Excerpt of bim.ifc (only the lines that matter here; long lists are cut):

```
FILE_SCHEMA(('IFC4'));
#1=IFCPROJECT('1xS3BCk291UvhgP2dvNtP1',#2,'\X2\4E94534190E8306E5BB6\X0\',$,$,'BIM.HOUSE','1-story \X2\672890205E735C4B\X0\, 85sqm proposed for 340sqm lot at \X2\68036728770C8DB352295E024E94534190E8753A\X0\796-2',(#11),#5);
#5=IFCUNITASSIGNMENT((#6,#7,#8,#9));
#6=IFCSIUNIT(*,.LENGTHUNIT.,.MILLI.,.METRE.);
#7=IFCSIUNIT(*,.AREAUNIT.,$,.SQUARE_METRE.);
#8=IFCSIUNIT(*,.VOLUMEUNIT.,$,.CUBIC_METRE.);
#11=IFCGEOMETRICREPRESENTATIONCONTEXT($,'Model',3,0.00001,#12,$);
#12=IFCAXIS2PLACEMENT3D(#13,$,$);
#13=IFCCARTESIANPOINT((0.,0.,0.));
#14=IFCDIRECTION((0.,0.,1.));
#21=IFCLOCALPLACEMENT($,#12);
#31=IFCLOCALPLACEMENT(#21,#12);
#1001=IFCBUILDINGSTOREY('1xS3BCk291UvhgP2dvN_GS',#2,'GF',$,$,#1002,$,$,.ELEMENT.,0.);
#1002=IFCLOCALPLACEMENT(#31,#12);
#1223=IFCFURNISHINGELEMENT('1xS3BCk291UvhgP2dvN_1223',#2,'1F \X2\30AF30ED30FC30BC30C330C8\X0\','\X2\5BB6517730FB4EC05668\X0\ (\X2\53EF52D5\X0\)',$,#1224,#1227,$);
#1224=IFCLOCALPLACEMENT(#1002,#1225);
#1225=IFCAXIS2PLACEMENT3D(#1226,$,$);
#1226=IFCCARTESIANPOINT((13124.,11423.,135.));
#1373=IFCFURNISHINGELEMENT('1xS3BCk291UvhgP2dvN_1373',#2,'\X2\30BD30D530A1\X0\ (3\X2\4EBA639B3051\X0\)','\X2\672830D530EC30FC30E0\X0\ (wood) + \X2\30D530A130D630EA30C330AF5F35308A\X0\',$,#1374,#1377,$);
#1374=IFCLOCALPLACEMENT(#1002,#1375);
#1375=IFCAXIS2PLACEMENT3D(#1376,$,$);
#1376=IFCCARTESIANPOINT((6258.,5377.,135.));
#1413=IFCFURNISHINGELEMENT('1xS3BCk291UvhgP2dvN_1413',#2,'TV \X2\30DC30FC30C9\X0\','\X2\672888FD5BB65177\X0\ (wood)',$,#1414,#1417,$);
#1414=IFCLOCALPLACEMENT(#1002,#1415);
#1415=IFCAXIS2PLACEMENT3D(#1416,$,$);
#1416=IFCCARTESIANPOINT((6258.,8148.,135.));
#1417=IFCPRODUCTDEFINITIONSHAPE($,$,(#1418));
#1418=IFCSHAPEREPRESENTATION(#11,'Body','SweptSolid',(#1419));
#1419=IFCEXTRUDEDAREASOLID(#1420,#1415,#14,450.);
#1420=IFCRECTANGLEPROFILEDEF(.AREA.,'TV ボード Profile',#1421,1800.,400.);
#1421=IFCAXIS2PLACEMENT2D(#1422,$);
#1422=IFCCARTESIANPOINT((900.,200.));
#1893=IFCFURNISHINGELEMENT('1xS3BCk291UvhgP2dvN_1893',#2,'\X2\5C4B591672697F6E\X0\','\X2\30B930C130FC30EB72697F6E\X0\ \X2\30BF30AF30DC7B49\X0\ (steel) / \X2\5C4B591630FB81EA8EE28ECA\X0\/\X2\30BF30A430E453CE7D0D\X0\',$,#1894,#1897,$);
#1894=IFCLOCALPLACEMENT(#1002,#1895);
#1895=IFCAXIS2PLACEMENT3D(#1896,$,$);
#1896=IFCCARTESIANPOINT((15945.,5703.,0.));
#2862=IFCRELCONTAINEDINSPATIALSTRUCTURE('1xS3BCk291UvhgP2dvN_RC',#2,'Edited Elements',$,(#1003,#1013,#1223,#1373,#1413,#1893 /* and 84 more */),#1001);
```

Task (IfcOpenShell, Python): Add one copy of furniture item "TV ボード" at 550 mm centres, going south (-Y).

```python
import numpy as np
import ifcopenshell
import ifcopenshell.api.geometry
import ifcopenshell.api.root
import ifcopenshell.util.element
import ifcopenshell.util.placement
import ifcopenshell.util.unit

model = ifcopenshell.open("bim.ifc")
unit_scale = ifcopenshell.util.unit.calculate_unit_scale(model)


def reuse_history(source, copy):
    """copy_class also copies each property set's owner history, people and application; keep the originals."""
    for rel in copy.IsDefinedBy:
        if rel.is_a("IfcRelDefinesByProperties") and (history := rel.RelatingPropertyDefinition.OwnerHistory):
            rel.RelatingPropertyDefinition.OwnerHistory = source.OwnerHistory
            ifcopenshell.util.element.remove_deep2(model, history)


source = model.by_guid("1xS3BCk291UvhgP2dvN_1413")
base = ifcopenshell.util.placement.get_local_placement(source.ObjectPlacement)
step = np.array([0.0, -1.0, 0.0]) * 0.55 / unit_scale

for i in range(1, 2):
    copy = ifcopenshell.api.root.copy_class(model, product=source)
    copy.Representation = ifcopenshell.util.element.copy_deep(
        model, source.Representation, exclude=["IfcGeometricRepresentationContext", "IfcRepresentationMap"]
    )
    reuse_history(source, copy)
    matrix = base.copy()
    matrix[:3, 3] += i * step
    print("added at", matrix[:3, 3].round(3) + 0.0)
    ifcopenshell.api.geometry.edit_object_placement(model, product=copy, matrix=matrix, is_si=False)

model.write("bim-out.ifc")
```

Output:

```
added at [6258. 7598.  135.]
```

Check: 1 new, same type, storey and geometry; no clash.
